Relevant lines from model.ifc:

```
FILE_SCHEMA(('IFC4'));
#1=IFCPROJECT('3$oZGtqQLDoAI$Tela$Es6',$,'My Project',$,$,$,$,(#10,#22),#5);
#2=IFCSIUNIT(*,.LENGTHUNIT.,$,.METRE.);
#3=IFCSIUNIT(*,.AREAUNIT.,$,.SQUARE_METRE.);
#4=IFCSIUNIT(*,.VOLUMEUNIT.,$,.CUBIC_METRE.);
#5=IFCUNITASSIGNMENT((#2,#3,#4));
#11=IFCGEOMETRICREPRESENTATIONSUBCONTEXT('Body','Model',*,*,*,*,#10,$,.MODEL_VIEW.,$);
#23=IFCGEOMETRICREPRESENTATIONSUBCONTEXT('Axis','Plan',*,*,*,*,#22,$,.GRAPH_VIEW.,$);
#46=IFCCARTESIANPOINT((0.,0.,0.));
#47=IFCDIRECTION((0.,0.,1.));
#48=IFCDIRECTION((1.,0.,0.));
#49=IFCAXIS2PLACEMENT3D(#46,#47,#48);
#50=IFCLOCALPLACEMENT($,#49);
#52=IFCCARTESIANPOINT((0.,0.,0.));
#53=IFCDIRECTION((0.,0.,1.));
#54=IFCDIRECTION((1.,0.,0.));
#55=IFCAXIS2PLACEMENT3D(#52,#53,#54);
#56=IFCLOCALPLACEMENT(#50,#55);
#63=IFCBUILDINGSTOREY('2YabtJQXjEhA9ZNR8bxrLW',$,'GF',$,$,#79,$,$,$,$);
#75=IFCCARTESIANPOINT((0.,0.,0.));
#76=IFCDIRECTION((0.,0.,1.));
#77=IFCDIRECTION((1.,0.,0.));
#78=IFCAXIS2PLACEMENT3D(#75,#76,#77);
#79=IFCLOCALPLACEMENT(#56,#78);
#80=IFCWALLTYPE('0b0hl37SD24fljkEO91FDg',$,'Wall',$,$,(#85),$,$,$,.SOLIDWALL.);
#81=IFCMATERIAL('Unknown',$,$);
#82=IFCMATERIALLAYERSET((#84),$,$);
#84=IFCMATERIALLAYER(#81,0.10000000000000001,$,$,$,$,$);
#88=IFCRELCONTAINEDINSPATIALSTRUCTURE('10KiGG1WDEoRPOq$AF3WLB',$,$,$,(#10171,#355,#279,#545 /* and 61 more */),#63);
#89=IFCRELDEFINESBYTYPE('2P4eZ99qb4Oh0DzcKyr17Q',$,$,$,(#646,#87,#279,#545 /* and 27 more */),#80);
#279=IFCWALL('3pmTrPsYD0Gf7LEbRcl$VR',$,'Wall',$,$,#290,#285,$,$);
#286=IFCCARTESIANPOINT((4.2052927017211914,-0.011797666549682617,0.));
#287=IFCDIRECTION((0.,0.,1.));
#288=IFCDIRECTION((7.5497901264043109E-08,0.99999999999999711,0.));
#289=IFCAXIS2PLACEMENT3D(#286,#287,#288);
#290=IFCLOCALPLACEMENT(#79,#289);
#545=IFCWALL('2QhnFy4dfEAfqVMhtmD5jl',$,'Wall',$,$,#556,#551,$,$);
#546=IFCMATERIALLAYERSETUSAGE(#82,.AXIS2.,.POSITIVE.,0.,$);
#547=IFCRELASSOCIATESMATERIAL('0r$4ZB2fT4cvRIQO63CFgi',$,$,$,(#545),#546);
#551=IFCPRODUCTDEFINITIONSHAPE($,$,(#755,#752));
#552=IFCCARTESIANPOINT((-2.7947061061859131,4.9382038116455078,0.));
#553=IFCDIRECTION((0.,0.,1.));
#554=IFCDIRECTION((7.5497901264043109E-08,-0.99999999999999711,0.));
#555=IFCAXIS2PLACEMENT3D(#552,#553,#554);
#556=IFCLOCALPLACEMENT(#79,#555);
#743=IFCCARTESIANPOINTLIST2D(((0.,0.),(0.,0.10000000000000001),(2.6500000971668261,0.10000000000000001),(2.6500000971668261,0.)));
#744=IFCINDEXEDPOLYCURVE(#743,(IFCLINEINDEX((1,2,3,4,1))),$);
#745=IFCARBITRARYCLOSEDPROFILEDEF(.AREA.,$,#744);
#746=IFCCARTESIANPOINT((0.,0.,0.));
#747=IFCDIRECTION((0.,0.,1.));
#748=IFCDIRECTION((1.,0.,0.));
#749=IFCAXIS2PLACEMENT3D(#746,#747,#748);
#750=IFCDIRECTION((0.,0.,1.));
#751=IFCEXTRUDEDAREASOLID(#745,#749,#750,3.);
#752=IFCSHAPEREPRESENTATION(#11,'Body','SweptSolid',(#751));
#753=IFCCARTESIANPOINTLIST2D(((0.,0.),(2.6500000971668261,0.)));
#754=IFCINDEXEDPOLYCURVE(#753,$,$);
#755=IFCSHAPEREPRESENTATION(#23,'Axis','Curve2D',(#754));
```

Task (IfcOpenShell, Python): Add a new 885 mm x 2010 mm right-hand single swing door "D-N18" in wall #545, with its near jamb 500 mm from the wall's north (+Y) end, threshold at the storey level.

```python
import numpy as np
import ifcopenshell
import ifcopenshell.api.feature
import ifcopenshell.api.geometry
import ifcopenshell.api.root
import ifcopenshell.api.spatial
import ifcopenshell.geom
import ifcopenshell.util.element
import ifcopenshell.util.placement
import ifcopenshell.util.representation
import ifcopenshell.util.shape
import ifcopenshell.util.unit

model = ifcopenshell.open("model.ifc")
unit_scale = ifcopenshell.util.unit.calculate_unit_scale(model)
settings = ifcopenshell.geom.settings()


def volume(element):
    """Net volume in cubic metres, openings subtracted."""
    shape = ifcopenshell.geom.create_shape(settings, element)
    return ifcopenshell.util.shape.get_volume(shape.geometry)


wall = model.by_id(545)
storey = ifcopenshell.util.element.get_container(wall, ifc_class="IfcBuildingStorey")
context = ifcopenshell.util.representation.get_context(model, "Model", "Body", "MODEL_VIEW")
before = volume(wall)

width, height, from_end, sill = 0.885, 2.01, 0.5, 0.0  # metres

# The wall runs along its own X axis, and the end named is its -X end.
wall_shape = ifcopenshell.geom.create_shape(settings, wall)
x, y, z = ifcopenshell.util.shape.get_vertices(wall_shape.geometry).T
start = x.min() + from_end
face, thickness = float(y.min()), float(y.max() - y.min())
wall_matrix = ifcopenshell.util.placement.get_local_placement(wall.ObjectPlacement)
level = ifcopenshell.util.placement.get_local_placement(storey.ObjectPlacement)[2, 3]


def in_wall(x, y):
    """Placement at x, y metres in the wall's axes, at sill height."""
    matrix = wall_matrix.copy()
    matrix[:, 3] = wall_matrix @ np.array([x / unit_scale, y / unit_scale, 0.0, 1.0])
    matrix[2, 3] = level + sill / unit_scale
    return matrix


# Opening: a box that overshoots both wall faces by 50 mm.
opening = ifcopenshell.api.root.create_entity(model, ifc_class="IfcOpeningElement", predefined_type="OPENING")
box = ifcopenshell.api.geometry.add_wall_representation(
    model, context=context, length=width, height=height, thickness=thickness + 0.1
)
ifcopenshell.api.geometry.assign_representation(model, product=opening, representation=box)
ifcopenshell.api.geometry.edit_object_placement(model, product=opening, matrix=in_wall(start, face - 0.05), is_si=False)
ifcopenshell.api.feature.add_feature(model, feature=opening, element=wall)

door = ifcopenshell.api.root.create_entity(model, ifc_class="IfcDoor", name="D-N18", predefined_type="DOOR")
door.OverallWidth, door.OverallHeight = width / unit_scale, height / unit_scale
door.OperationType = "SINGLE_SWING_RIGHT"
body = ifcopenshell.api.geometry.add_door_representation(
    model,
    context=context,
    overall_width=door.OverallWidth,
    overall_height=door.OverallHeight,
    operation_type="SINGLE_SWING_RIGHT",
    lining_properties={"LiningDepth": thickness / unit_scale, "ThresholdDepth": thickness / unit_scale},
)
ifcopenshell.api.geometry.assign_representation(model, product=door, representation=body)
ifcopenshell.api.spatial.assign_container(model, products=[door], relating_structure=storey)
ifcopenshell.api.feature.add_filling(model, opening=opening, element=door)

# The lining spans the wall, so the door starts at the wall face.
ifcopenshell.api.geometry.edit_object_placement(model, product=door, matrix=in_wall(start, face), is_si=False)

after = volume(wall)

print(f"wall volume {before:.3f} -> {after:.3f} m3")

model.write("model_updated.ifc")
```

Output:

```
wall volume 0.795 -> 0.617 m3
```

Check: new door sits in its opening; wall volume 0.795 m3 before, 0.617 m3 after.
